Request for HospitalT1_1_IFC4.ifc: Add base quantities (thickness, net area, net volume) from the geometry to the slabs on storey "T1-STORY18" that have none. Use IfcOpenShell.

First a look at what the model holds.

```python
import ifcopenshell
import ifcopenshell.util.element
import ifcopenshell.util.unit

model = ifcopenshell.open("HospitalT1_1_IFC4.ifc")
print(model.schema)
for unit_type in ("LENGTHUNIT", "AREAUNIT", "VOLUMEUNIT"):
    print(unit_type, ifcopenshell.util.unit.calculate_unit_scale(model, unit_type))
storey = next(s for s in model.by_type("IfcBuildingStorey") if s.Name == "T1-STORY18")
slabs = [e for e in ifcopenshell.util.element.get_decomposition(storey) if e.is_a("IfcSlab")]
for e in sorted(slabs, key=lambda e: e.id()):
    print(e.id(), e.is_a(), e.Name, list(ifcopenshell.util.element.get_psets(e, qtos_only=True)), sep=" | ")
```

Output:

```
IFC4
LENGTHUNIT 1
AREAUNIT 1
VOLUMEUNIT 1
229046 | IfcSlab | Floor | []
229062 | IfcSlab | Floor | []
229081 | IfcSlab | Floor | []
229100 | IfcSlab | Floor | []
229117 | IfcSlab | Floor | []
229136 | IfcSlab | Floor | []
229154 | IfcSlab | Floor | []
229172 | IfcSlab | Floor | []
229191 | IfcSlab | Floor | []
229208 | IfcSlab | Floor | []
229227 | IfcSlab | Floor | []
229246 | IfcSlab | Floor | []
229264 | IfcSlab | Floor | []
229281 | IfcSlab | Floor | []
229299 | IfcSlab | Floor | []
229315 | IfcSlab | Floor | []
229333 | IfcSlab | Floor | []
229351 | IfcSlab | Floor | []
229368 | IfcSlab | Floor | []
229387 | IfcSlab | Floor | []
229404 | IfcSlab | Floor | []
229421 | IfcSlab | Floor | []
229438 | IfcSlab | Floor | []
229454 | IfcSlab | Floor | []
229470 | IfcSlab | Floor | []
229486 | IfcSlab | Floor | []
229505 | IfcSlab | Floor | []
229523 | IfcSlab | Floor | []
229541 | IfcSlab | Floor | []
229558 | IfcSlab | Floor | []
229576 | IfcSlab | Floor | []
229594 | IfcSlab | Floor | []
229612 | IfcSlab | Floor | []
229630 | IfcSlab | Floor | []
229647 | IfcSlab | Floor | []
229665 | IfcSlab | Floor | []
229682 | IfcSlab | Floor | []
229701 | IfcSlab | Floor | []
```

```python
import ifcopenshell
import ifcopenshell.api.pset
import ifcopenshell.geom
import ifcopenshell.util.element
import ifcopenshell.util.shape
import ifcopenshell.util.unit

model = ifcopenshell.open("HospitalT1_1_IFC4.ifc")
unit_scale = ifcopenshell.util.unit.calculate_unit_scale(model)
area_scale = ifcopenshell.util.unit.calculate_unit_scale(model, "AREAUNIT")
volume_scale = ifcopenshell.util.unit.calculate_unit_scale(model, "VOLUMEUNIT")
settings = ifcopenshell.geom.settings()

storey = next(s for s in model.by_type("IfcBuildingStorey") if s.Name == "T1-STORY18")
slabs = [e for e in ifcopenshell.util.element.get_decomposition(storey) if e.is_a("IfcSlab")]

for e in sorted(slabs, key=lambda e: e.id()):
    if ifcopenshell.util.element.get_psets(e, qtos_only=True, should_inherit=False):
        continue
    # Geometry comes back in metres, in the element's own axes.
    shape = ifcopenshell.geom.create_shape(settings, e)
    values = {
        "Width": ifcopenshell.util.shape.get_z(shape.geometry) / unit_scale,
        "NetArea": ifcopenshell.util.shape.get_footprint_area(shape.geometry) / area_scale,
        "NetVolume": ifcopenshell.util.shape.get_volume(shape.geometry) / volume_scale,
    }
    qto = ifcopenshell.api.pset.add_qto(model, product=e, name="Qto_SlabBaseQuantities")
    ifcopenshell.api.pset.edit_qto(model, qto=qto, properties=values)
    print(e.id(), {k: round(v, 3) for k, v in values.items()})

model.write("HospitalT1_1_IFC4_edited.ifc")
```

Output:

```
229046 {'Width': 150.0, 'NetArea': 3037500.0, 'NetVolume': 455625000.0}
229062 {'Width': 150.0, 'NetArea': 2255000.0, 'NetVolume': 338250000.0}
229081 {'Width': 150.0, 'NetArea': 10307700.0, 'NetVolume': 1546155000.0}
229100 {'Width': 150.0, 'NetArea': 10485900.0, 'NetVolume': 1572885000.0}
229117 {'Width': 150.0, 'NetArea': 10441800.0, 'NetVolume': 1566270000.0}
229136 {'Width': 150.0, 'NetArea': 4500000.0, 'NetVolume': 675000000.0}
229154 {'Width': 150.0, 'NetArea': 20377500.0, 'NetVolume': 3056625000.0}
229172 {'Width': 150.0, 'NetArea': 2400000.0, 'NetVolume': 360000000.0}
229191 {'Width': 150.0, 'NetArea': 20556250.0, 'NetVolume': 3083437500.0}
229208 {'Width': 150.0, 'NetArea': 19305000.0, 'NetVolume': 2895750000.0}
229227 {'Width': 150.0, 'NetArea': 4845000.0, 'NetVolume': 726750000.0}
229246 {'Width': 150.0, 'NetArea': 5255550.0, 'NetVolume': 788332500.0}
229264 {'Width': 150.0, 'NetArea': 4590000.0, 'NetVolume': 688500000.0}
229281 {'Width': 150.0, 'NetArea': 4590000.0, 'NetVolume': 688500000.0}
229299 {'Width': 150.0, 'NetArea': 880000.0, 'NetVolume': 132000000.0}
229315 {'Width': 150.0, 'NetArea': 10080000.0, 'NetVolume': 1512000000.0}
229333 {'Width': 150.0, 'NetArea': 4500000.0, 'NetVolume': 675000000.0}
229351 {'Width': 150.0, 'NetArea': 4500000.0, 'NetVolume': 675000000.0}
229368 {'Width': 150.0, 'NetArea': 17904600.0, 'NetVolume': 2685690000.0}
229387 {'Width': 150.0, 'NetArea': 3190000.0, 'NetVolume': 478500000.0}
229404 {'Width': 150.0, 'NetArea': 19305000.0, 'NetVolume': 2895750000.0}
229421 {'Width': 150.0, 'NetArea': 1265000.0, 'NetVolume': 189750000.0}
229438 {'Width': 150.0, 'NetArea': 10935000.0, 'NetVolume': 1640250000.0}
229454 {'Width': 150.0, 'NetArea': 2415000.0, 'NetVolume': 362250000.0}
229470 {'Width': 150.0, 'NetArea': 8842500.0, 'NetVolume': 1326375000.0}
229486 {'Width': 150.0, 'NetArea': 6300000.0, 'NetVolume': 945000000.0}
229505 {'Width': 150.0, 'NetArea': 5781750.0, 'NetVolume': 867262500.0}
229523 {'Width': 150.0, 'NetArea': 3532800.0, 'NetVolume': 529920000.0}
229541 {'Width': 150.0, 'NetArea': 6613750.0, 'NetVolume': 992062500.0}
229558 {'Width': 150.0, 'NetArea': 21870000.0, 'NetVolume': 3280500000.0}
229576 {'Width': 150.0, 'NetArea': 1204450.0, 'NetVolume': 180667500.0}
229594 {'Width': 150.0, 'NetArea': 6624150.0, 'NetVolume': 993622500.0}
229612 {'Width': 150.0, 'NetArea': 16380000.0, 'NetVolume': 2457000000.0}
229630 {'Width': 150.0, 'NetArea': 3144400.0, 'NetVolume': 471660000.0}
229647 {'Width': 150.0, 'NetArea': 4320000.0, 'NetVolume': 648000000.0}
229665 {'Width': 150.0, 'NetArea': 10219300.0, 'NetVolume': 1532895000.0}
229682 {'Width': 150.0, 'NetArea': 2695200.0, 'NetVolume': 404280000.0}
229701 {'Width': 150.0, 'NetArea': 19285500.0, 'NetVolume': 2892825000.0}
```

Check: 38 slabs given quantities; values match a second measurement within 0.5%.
